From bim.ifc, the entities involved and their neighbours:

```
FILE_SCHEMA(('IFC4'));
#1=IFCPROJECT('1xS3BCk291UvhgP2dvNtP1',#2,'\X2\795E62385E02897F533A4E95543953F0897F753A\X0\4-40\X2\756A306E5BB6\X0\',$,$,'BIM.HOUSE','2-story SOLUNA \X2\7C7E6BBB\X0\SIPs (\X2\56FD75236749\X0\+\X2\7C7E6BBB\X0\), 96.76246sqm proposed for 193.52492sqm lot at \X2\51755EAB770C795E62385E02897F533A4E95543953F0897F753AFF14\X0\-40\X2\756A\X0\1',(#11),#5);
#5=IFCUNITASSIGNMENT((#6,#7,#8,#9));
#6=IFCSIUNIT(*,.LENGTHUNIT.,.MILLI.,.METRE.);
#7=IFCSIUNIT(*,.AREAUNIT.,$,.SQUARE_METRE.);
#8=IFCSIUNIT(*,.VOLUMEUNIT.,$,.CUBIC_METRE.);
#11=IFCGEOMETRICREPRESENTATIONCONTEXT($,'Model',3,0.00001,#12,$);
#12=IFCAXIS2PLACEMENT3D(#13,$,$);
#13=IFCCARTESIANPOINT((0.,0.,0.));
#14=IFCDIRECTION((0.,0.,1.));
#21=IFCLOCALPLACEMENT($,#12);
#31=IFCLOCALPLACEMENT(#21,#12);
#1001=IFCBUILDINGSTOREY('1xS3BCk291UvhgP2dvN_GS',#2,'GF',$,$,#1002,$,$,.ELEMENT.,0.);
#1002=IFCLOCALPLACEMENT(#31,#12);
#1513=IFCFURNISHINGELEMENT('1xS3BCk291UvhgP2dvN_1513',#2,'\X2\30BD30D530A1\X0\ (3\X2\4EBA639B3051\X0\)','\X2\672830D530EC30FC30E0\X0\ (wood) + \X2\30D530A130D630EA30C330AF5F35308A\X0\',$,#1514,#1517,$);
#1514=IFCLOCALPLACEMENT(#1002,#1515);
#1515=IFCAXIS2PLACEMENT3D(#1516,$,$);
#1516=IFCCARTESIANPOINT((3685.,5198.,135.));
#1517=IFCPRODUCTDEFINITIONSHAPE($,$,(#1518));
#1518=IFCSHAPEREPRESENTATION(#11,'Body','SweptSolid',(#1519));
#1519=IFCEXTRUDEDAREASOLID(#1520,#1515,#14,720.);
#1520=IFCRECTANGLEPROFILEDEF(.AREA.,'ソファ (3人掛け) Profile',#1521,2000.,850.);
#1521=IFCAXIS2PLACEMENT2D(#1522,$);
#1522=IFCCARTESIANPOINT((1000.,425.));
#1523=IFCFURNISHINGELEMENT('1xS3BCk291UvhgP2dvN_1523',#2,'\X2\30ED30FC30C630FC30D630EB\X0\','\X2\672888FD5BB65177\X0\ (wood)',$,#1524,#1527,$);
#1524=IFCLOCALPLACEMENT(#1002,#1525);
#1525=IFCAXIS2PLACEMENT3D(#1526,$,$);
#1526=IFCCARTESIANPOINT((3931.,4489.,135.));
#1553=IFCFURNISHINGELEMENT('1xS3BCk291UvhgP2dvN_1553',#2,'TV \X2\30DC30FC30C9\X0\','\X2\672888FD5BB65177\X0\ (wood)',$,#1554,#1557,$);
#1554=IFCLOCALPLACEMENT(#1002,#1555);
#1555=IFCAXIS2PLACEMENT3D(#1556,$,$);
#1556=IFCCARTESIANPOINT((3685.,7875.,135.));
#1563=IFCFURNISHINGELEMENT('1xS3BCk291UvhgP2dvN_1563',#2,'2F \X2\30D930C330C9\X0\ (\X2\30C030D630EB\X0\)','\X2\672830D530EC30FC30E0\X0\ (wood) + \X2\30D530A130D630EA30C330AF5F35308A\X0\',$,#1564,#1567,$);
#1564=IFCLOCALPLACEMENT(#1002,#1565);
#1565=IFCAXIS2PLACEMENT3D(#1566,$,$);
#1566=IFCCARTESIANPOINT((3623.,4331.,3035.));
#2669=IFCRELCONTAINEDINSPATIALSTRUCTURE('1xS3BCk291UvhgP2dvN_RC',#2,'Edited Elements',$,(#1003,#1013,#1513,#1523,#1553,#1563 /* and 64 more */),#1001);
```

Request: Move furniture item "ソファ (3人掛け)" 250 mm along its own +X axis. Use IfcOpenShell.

```python
import ifcopenshell
import ifcopenshell.api.geometry
import ifcopenshell.util.placement
import ifcopenshell.util.unit

model = ifcopenshell.open("bim.ifc")
unit_scale = ifcopenshell.util.unit.calculate_unit_scale(model)

item = model.by_guid("1xS3BCk291UvhgP2dvN_1513")
matrix = ifcopenshell.util.placement.get_local_placement(item.ObjectPlacement)
matrix[:3, 3] += matrix[:3, 0] * 0.25 / unit_scale
ifcopenshell.api.geometry.edit_object_placement(model, product=item, matrix=matrix, is_si=False)

print(ifcopenshell.util.placement.get_local_placement(item.ObjectPlacement).round(3) + 0.0)

model.write("bim_v2.ifc")
```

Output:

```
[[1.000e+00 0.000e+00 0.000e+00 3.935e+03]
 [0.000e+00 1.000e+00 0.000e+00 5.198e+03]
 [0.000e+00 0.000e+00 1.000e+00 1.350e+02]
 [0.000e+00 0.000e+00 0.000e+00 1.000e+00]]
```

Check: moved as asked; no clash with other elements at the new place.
